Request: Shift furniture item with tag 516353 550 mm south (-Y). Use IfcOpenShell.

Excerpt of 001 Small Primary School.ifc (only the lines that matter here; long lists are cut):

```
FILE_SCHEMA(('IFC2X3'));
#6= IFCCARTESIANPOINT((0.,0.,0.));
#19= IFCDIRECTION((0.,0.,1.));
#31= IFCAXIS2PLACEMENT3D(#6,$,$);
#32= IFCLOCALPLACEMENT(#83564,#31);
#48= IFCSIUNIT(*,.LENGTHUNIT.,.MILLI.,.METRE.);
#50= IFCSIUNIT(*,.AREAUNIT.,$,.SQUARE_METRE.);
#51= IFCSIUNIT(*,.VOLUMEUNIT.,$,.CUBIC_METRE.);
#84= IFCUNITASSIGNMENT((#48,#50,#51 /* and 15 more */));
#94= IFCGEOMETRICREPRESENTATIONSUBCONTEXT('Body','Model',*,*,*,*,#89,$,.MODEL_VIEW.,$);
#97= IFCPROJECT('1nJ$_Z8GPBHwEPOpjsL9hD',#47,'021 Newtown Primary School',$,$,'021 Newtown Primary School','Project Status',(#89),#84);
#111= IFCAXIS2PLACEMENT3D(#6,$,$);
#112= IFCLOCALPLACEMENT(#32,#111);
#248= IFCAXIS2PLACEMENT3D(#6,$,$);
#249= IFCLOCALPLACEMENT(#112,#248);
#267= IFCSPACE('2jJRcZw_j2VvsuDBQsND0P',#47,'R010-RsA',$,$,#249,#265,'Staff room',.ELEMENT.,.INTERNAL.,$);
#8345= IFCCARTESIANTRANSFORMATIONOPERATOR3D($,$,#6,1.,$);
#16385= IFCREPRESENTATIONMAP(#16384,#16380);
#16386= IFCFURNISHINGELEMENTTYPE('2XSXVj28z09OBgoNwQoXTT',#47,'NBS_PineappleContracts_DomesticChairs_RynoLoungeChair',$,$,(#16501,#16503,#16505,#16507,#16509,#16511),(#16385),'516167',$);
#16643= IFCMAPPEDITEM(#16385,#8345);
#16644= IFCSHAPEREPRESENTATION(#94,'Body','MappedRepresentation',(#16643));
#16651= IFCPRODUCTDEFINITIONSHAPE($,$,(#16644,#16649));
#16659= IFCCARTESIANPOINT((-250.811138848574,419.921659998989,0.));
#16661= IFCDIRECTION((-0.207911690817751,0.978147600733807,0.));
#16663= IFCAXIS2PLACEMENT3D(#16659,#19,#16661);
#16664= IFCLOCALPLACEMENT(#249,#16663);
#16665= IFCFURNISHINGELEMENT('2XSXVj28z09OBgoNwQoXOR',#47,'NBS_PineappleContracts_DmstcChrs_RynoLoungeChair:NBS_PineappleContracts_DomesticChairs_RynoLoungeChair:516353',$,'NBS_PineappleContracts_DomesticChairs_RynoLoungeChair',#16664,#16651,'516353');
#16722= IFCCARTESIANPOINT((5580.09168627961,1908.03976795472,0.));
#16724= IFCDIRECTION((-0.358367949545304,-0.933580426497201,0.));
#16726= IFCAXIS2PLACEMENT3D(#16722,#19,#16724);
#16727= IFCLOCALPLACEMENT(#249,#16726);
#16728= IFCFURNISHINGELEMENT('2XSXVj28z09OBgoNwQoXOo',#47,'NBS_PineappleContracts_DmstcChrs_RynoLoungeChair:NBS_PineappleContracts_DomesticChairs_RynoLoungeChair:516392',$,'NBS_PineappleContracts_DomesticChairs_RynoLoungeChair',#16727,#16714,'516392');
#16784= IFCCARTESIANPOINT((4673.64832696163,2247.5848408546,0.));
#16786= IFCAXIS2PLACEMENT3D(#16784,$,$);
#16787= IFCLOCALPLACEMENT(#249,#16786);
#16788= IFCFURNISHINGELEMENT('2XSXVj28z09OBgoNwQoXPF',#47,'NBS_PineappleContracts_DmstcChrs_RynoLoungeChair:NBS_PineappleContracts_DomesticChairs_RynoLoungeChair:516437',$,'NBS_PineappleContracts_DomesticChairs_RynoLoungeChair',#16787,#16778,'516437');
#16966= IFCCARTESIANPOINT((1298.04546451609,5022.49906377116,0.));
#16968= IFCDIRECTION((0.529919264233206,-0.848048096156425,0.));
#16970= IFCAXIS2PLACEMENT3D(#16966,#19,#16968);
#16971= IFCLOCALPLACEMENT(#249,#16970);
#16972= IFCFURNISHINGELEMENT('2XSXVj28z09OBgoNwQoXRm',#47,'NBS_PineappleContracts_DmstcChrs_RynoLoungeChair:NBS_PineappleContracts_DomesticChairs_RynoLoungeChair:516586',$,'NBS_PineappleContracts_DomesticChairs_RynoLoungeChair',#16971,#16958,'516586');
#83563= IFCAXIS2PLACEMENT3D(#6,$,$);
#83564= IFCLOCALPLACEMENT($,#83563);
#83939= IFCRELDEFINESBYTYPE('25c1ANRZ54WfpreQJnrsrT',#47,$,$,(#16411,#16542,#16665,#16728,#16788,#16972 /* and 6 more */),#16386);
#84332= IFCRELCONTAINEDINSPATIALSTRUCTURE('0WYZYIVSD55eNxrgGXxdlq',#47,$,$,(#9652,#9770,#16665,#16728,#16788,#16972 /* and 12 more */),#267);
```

```python
import ifcopenshell
import ifcopenshell.api.geometry
import ifcopenshell.util.placement

model = ifcopenshell.open("001 Small Primary School.ifc")

item = model.by_guid("2XSXVj28z09OBgoNwQoXOR")
matrix = ifcopenshell.util.placement.get_local_placement(item.ObjectPlacement)
matrix[1, 3] -= 550.0
ifcopenshell.api.geometry.edit_object_placement(model, product=item, matrix=matrix, is_si=False)

print(ifcopenshell.util.placement.get_local_placement(item.ObjectPlacement).round(3) + 0.0)

model.write("001 Small Primary School_rev.ifc")
```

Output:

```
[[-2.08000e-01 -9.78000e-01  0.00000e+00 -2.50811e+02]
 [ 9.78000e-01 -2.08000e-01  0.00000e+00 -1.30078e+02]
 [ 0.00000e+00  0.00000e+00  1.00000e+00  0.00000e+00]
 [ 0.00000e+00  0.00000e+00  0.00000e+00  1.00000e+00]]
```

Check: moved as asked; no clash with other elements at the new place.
